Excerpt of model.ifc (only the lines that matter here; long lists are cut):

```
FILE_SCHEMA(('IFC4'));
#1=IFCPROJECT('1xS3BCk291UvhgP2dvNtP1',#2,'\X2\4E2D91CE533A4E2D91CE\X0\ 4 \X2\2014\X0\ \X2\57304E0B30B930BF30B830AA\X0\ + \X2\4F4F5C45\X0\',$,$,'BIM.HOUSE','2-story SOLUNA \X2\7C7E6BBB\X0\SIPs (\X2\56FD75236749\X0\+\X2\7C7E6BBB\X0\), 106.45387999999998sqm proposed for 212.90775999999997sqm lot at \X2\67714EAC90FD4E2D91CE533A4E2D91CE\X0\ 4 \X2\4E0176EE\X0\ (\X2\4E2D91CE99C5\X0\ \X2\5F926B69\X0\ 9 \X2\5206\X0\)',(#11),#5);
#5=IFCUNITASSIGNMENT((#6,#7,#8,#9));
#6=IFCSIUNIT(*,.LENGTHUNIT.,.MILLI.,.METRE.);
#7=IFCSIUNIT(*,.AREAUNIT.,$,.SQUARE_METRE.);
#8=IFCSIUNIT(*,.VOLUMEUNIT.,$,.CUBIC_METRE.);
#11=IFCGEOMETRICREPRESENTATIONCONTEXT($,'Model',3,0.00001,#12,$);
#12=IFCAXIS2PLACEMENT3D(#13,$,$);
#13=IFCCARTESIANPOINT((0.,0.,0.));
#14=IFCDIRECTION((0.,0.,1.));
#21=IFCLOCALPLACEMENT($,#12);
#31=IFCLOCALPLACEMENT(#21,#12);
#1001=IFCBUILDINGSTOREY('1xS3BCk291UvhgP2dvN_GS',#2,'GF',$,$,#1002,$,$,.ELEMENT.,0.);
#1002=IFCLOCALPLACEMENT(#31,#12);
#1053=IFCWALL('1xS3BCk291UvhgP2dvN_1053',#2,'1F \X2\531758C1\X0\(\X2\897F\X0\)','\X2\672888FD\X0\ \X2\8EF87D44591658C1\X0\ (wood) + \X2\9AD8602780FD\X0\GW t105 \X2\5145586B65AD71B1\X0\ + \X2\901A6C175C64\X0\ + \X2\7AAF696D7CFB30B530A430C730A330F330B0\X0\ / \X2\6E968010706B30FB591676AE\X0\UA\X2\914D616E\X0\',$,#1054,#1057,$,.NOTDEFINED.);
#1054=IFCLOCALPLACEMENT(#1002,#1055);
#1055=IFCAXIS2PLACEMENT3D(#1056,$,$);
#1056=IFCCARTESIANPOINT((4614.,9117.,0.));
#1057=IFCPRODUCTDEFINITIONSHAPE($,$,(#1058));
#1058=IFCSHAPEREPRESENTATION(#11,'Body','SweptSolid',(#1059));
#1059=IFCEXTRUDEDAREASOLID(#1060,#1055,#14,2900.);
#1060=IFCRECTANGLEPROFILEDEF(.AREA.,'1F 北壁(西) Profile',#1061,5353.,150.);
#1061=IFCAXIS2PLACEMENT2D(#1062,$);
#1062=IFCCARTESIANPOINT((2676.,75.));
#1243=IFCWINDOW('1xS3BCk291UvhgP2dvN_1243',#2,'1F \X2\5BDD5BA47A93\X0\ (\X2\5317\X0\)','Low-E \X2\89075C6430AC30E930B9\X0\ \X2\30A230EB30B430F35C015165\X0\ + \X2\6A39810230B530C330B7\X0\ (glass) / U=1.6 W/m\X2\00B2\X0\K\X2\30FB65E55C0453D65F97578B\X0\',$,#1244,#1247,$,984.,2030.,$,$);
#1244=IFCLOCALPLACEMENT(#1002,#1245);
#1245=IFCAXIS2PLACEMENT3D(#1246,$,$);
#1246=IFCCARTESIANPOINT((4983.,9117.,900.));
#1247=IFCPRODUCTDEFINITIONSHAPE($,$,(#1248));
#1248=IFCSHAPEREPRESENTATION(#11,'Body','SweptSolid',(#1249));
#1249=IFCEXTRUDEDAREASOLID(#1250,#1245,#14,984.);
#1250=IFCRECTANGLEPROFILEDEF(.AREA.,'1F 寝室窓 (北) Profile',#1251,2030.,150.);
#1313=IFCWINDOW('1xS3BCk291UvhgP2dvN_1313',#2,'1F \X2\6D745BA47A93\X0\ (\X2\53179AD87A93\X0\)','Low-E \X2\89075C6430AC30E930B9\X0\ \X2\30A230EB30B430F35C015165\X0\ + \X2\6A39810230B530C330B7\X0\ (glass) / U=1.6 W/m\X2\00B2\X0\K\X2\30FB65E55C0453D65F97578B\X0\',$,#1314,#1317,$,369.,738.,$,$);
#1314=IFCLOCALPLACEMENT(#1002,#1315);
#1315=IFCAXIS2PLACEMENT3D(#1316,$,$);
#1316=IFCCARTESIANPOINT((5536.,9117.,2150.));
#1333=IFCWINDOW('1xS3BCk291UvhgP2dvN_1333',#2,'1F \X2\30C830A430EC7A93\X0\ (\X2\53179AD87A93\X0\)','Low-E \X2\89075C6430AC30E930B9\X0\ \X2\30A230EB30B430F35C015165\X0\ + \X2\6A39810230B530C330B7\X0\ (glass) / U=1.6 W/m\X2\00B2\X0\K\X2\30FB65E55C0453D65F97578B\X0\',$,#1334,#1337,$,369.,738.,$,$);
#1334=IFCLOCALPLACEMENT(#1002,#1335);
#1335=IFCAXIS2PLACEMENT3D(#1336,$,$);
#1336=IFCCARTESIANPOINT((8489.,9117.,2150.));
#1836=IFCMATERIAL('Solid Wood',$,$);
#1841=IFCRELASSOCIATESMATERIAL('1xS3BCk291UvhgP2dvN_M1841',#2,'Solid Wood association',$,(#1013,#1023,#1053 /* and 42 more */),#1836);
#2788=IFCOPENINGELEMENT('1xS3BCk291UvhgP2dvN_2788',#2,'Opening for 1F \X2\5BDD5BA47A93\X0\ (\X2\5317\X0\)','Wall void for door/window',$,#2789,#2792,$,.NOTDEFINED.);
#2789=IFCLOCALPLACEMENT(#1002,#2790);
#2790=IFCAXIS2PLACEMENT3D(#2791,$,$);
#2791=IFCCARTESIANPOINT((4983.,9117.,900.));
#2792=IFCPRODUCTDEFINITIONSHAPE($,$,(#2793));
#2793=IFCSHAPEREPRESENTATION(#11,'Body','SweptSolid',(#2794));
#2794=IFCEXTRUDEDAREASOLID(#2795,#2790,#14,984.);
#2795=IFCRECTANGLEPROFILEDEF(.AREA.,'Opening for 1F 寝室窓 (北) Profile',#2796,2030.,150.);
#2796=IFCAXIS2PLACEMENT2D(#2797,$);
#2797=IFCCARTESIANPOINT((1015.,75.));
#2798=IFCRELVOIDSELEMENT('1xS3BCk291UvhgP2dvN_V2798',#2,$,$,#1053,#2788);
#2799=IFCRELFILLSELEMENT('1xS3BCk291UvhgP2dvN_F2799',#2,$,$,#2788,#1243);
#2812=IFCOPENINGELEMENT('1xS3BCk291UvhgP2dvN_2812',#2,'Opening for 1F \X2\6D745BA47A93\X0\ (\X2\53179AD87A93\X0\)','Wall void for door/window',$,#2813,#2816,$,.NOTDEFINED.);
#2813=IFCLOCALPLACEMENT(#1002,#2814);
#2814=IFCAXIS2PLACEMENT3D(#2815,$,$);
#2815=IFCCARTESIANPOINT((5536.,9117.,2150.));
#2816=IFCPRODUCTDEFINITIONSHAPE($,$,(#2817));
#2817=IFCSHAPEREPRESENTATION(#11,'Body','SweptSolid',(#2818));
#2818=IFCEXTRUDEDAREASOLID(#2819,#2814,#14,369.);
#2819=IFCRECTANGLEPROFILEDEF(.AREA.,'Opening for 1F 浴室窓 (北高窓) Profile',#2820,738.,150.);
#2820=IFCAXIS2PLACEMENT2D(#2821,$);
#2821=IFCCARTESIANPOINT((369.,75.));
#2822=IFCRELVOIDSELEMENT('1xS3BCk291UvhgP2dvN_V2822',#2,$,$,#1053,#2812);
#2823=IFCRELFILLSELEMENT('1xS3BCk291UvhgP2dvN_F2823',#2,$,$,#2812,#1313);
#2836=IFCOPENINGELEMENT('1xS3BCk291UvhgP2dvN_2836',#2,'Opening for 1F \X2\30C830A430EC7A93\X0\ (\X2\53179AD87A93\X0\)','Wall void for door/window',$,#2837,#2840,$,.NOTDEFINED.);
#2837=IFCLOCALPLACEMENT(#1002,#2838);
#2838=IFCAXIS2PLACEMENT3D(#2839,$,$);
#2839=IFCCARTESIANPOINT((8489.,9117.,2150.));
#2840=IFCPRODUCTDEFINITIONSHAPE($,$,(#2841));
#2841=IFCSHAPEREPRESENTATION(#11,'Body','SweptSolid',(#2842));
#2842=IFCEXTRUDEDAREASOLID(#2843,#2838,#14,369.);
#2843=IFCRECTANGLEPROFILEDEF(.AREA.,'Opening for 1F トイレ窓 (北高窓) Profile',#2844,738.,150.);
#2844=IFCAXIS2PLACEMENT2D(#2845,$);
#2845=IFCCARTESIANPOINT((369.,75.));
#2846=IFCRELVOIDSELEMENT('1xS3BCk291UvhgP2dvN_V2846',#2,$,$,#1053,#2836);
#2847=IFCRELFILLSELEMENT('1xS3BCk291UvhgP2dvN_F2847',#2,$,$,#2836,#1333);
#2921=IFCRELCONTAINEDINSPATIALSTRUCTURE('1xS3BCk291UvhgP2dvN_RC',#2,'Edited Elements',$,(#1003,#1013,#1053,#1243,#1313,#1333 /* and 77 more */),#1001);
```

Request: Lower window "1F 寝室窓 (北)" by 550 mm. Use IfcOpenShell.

```python
import numpy as np
import ifcopenshell
import ifcopenshell.api.geometry
import ifcopenshell.util.placement
import ifcopenshell.util.unit

model = ifcopenshell.open("model.ifc")
unit_scale = ifcopenshell.util.unit.calculate_unit_scale(model)

window = model.by_guid("1xS3BCk291UvhgP2dvN_1243")
opening = window.FillsVoids[0].RelatingOpeningElement
dz = -0.55 / unit_scale

shift = np.array([0.0, 0.0, dz])
# The window is not placed relative to its opening, so move both.
for product in (opening, window):
    matrix = ifcopenshell.util.placement.get_local_placement(product.ObjectPlacement)
    matrix[:3, 3] += shift
    ifcopenshell.api.geometry.edit_object_placement(model, product=product, matrix=matrix, is_si=False)

print(f"moved by {dz * unit_scale:+.3f} m")

model.write("model_updated.ifc")
```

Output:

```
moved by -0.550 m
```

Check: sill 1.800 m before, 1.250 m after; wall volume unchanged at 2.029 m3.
